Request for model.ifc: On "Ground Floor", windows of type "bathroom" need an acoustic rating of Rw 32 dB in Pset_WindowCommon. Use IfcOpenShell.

First a look at what the model holds.

```python
import ifcopenshell
import ifcopenshell.util.element

model = ifcopenshell.open("model.ifc")
print(model.schema)
storey = next(s for s in model.by_type("IfcBuildingStorey") if s.Name == "Ground Floor")
windows = [e for e in ifcopenshell.util.element.get_decomposition(storey) if e.is_a("IfcWindow")]
seen = {}
for e in windows:
    element_type = ifcopenshell.util.element.get_type(e)
    key = (element_type.Name if element_type != e and element_type else None, ifcopenshell.util.element.get_pset(e, "Pset_WindowCommon", "AcousticRating"))
    seen[key] = seen.get(key, 0) + 1
for (name, value), count in sorted(seen.items(), key=str):
    print(count, "x", name, "|", value)
```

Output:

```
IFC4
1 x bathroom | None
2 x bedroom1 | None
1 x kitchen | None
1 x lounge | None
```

```python
import ifcopenshell
import ifcopenshell.api.pset
import ifcopenshell.util.element

model = ifcopenshell.open("model.ifc")

storey = next(s for s in model.by_type("IfcBuildingStorey") if s.Name == "Ground Floor")
windows = [e for e in ifcopenshell.util.element.get_decomposition(storey) if e.is_a("IfcWindow")]

count = 0
for e in windows:
    element_type = ifcopenshell.util.element.get_type(e)
    if element_type in (None, e) or element_type.Name != "bathroom":
        continue
    # add_pset returns the element's existing set when there is one.
    pset = ifcopenshell.api.pset.add_pset(model, product=e, name="Pset_WindowCommon")
    ifcopenshell.api.pset.edit_pset(model, pset=pset, properties={"AcousticRating": "Rw 32 dB"})
    count += 1

print(count, "windows updated")

model.write("model_v2.ifc")
```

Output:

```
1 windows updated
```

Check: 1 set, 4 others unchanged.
